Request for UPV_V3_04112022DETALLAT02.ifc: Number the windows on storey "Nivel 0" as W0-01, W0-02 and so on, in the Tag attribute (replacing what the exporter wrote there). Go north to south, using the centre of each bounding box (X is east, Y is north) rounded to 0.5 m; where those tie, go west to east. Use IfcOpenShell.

First a look at what the model holds.

```python
import ifcopenshell
import ifcopenshell.util.element
import ifcopenshell.util.placement

model = ifcopenshell.open("UPV_V3_04112022DETALLAT02.ifc")
print(model.schema)
storey = next(s for s in model.by_type("IfcBuildingStorey") if s.Name == "Nivel 0")
windows = [e for e in ifcopenshell.util.element.get_decomposition(storey) if e.is_a("IfcWindow")]
for e in sorted(windows, key=lambda e: e.id()):
    origin = ifcopenshell.util.placement.get_local_placement(e.ObjectPlacement)[:3, 3]
    print(e.id(), e.Tag, e.Name, origin.round(2) + 0.0, sep=" | ")
```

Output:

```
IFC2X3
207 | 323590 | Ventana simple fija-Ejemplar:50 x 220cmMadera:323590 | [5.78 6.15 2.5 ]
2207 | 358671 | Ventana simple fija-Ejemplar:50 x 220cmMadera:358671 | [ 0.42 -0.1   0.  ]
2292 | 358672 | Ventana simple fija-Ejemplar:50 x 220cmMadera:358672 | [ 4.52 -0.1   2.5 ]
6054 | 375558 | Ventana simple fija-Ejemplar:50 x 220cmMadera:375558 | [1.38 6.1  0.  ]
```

```python
import ifcopenshell
import ifcopenshell.geom
import ifcopenshell.util.element
import ifcopenshell.util.shape

model = ifcopenshell.open("UPV_V3_04112022DETALLAT02.ifc")
settings = ifcopenshell.geom.settings()
settings.set("use-world-coords", True)


def centre(element):
    shape = ifcopenshell.geom.create_shape(settings, element)
    return ifcopenshell.util.shape.get_bbox_centroid(shape.geometry)


storey = next(s for s in model.by_type("IfcBuildingStorey") if s.Name == "Nivel 0")
windows = [e for e in ifcopenshell.util.element.get_decomposition(storey) if e.is_a("IfcWindow")]

# Insertion points can sit at a corner or the storey origin, so sort by the geometry (in metres).
centres = {e: centre(e) for e in windows}
windows.sort(key=lambda e: (-round(centres[e][1] / 0.5), centres[e][0]))

for i, e in enumerate(windows, start=1):
    number = f"W0-{i:02d}"
    e.Tag = number
    print(e.id(), number)

model.write("UPV_V3_04112022DETALLAT02_edited.ifc")
```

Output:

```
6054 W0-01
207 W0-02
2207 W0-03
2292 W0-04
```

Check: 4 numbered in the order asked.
